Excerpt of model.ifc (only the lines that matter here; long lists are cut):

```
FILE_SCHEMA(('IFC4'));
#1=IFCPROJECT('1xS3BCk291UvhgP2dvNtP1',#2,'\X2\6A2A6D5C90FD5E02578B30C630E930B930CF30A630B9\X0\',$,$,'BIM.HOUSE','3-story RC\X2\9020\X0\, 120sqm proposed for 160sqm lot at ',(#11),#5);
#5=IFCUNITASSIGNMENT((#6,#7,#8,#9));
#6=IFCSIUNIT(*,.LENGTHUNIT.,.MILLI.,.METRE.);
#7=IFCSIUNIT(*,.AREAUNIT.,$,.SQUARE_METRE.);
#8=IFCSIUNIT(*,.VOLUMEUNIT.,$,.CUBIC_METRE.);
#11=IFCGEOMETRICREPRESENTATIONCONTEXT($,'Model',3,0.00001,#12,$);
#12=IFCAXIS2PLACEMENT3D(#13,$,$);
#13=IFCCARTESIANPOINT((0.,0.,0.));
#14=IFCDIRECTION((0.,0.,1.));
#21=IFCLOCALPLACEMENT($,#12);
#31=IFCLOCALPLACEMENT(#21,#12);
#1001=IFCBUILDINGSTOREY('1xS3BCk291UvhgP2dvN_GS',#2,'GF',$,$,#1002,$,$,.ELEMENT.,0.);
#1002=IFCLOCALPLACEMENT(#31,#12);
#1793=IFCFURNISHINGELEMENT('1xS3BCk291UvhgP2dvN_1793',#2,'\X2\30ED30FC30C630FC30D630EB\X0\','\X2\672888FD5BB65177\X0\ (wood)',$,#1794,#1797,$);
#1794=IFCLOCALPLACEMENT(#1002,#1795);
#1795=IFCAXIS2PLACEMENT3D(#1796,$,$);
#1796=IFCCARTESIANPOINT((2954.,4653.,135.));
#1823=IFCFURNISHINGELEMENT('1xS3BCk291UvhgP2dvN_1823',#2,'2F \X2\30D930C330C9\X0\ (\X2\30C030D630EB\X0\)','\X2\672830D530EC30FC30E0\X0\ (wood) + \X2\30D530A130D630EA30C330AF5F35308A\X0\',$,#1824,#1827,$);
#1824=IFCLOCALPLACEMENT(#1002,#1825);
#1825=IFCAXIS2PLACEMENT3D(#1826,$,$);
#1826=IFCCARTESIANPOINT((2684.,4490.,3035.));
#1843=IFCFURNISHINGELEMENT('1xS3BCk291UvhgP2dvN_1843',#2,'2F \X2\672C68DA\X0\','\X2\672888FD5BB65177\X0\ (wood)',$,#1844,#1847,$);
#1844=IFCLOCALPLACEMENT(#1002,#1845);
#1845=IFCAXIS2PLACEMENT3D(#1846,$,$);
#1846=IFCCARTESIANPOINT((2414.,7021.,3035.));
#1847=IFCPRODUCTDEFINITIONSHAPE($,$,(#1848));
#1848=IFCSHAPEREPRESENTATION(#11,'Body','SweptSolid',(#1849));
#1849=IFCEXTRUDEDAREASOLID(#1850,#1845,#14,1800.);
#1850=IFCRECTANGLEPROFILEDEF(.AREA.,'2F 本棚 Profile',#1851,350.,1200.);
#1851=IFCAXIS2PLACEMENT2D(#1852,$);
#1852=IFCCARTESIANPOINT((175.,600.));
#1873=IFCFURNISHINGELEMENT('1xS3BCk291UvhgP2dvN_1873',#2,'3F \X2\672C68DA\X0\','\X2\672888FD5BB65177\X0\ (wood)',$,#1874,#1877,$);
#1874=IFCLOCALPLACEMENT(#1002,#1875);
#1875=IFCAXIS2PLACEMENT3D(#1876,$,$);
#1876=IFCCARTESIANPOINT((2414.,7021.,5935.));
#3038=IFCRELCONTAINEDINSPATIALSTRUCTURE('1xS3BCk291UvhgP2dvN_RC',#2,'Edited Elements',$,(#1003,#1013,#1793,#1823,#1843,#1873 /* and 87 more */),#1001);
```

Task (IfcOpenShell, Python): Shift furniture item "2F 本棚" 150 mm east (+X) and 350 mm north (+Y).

```python
import ifcopenshell
import ifcopenshell.api.geometry
import ifcopenshell.util.placement
import ifcopenshell.util.unit

model = ifcopenshell.open("model.ifc")
unit_scale = ifcopenshell.util.unit.calculate_unit_scale(model)

item = model.by_guid("1xS3BCk291UvhgP2dvN_1843")
matrix = ifcopenshell.util.placement.get_local_placement(item.ObjectPlacement)
matrix[0, 3] += 0.15 / unit_scale
matrix[1, 3] += 0.35 / unit_scale
ifcopenshell.api.geometry.edit_object_placement(model, product=item, matrix=matrix, is_si=False)

print(ifcopenshell.util.placement.get_local_placement(item.ObjectPlacement).round(3) + 0.0)

model.write("model_v2.ifc")
```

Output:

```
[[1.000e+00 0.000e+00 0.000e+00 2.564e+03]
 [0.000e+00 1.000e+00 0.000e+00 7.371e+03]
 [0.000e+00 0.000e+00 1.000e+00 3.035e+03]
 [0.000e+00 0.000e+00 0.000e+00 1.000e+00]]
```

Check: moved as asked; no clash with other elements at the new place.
